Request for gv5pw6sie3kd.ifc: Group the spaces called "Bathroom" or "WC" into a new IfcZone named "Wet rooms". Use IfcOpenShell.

First a look at what the model holds.

```python
import ifcopenshell

model = ifcopenshell.open("gv5pw6sie3kd.ifc")
print(model.schema)
seen = {}
for space in model.by_type("IfcSpace"):
    seen[space.Name] = seen.get(space.Name, 0) + 1
for name, count in sorted(seen.items(), key=str):
    print(count, "x", name)
print("zones:", [z.Name for z in model.by_type("IfcZone")][:20])
```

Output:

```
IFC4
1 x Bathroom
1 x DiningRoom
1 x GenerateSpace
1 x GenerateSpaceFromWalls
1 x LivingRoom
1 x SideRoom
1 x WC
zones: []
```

```python
import ifcopenshell
import ifcopenshell.api.group
import ifcopenshell.api.root

model = ifcopenshell.open("gv5pw6sie3kd.ifc")

names = {"Bathroom", "WC"}
spaces = [s for s in model.by_type("IfcSpace") if s.Name in names]

zone = ifcopenshell.api.root.create_entity(model, ifc_class="IfcZone", name="Wet rooms")
ifcopenshell.api.group.assign_group(model, products=spaces, group=zone)
print(len(spaces), "spaces in", zone.Name)

model.write("gv5pw6sie3kd_v2.ifc")
```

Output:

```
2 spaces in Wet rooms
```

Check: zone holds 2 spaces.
